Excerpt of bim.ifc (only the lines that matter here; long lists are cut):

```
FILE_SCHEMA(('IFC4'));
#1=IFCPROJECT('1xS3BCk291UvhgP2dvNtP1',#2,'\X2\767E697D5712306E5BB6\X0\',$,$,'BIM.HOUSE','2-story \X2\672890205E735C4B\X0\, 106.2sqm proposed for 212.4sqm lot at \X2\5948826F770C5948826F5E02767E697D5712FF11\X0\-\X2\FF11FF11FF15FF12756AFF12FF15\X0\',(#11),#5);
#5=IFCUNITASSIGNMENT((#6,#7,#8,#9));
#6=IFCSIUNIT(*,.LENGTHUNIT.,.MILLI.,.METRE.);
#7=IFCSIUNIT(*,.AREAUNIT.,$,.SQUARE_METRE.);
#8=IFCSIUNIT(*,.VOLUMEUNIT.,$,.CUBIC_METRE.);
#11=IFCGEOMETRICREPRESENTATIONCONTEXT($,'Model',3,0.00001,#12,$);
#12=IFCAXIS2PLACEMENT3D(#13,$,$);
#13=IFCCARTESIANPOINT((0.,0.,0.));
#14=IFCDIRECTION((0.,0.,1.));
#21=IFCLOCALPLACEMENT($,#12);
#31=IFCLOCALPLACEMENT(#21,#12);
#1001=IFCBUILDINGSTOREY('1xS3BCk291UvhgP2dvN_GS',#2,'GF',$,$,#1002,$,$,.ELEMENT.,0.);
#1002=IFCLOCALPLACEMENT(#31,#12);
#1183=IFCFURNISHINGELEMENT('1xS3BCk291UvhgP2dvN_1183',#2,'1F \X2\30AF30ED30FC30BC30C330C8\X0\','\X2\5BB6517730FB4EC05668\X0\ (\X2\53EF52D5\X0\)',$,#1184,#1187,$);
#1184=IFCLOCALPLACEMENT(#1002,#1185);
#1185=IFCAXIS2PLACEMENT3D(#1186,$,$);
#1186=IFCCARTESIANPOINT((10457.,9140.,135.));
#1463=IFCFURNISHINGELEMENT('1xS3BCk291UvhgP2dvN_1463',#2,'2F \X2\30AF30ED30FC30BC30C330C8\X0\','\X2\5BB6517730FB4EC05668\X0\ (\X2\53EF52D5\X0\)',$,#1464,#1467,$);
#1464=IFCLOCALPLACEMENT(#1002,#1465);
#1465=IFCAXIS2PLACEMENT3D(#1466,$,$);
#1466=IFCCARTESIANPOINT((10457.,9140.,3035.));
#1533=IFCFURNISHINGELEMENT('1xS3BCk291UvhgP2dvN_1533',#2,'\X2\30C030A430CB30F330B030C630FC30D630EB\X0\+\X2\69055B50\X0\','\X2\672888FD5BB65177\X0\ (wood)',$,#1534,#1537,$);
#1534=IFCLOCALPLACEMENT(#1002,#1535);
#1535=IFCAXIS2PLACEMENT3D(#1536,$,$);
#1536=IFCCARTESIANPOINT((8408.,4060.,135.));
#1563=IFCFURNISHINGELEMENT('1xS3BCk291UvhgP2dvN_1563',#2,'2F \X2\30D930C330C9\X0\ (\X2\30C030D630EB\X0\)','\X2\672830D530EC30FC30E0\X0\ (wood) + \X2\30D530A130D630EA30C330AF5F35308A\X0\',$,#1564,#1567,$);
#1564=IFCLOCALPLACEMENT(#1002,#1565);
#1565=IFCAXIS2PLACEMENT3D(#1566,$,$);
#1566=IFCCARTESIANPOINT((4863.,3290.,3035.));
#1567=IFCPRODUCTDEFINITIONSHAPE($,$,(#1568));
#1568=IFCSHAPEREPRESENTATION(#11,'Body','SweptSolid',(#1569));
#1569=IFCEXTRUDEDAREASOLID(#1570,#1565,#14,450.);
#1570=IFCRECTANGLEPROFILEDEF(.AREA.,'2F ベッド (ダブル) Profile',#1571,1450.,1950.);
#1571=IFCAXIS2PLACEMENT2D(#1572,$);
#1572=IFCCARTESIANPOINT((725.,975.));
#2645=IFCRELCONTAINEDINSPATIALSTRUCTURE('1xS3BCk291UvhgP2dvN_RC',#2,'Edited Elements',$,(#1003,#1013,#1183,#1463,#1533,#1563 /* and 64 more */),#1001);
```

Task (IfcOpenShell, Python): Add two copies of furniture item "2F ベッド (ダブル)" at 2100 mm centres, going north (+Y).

```python
import numpy as np
import ifcopenshell
import ifcopenshell.api.geometry
import ifcopenshell.api.root
import ifcopenshell.util.element
import ifcopenshell.util.placement

model = ifcopenshell.open("bim.ifc")


def reuse_history(source, copy):
    """copy_class also copies each property set's owner history, people and application; keep the originals."""
    for rel in copy.IsDefinedBy:
        if rel.is_a("IfcRelDefinesByProperties") and (history := rel.RelatingPropertyDefinition.OwnerHistory):
            rel.RelatingPropertyDefinition.OwnerHistory = source.OwnerHistory
            ifcopenshell.util.element.remove_deep2(model, history)


source = model.by_id(1563)
base = ifcopenshell.util.placement.get_local_placement(source.ObjectPlacement)
step = np.array([0.0, 1.0, 0.0]) * 2100.0

for i in range(1, 3):
    copy = ifcopenshell.api.root.copy_class(model, product=source)
    copy.Representation = ifcopenshell.util.element.copy_deep(
        model, source.Representation, exclude=["IfcGeometricRepresentationContext", "IfcRepresentationMap"]
    )
    reuse_history(source, copy)
    matrix = base.copy()
    matrix[:3, 3] += i * step
    print("added at", matrix[:3, 3].round(3) + 0.0)
    ifcopenshell.api.geometry.edit_object_placement(model, product=copy, matrix=matrix, is_si=False)

model.write("bim_updated.ifc")
```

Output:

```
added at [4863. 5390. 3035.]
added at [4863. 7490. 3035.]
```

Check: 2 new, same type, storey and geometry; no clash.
